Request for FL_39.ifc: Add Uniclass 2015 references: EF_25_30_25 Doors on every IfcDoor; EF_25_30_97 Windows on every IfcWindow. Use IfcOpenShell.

First a look at what the model holds.

```python
import ifcopenshell

model = ifcopenshell.open("FL_39.ifc")
print(model.schema)
print("classifications:", [c.Name for c in model.by_type("IfcClassification")])
for ifc_class in ("IfcDoor", "IfcRoof", "IfcStair", "IfcWall", "IfcWindow"):
    print(ifc_class, len(model.by_type(ifc_class)))
```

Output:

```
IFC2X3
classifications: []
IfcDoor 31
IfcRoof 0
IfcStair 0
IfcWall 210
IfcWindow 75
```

```python
import ifcopenshell
import ifcopenshell.api.classification

model = ifcopenshell.open("FL_39.ifc")

# IFC2X3 requires Source and Edition and has no link from the project to the system.
system = model.create_entity("IfcClassification", Source="NBS", Edition="2015", Name="Uniclass 2015")

codes = {
    "IfcDoor": ("EF_25_30_25", "Doors"),
    "IfcWindow": ("EF_25_30_97", "Windows"),
}
for ifc_class, (code, name) in codes.items():
    products = model.by_type(ifc_class)
    ifcopenshell.api.classification.add_reference(
        model, products=products, classification=system, identification=code, name=name
    )
    print(code, len(products))

model.write("FL_39_edited.ifc")
```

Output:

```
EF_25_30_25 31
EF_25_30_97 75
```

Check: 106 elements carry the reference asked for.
